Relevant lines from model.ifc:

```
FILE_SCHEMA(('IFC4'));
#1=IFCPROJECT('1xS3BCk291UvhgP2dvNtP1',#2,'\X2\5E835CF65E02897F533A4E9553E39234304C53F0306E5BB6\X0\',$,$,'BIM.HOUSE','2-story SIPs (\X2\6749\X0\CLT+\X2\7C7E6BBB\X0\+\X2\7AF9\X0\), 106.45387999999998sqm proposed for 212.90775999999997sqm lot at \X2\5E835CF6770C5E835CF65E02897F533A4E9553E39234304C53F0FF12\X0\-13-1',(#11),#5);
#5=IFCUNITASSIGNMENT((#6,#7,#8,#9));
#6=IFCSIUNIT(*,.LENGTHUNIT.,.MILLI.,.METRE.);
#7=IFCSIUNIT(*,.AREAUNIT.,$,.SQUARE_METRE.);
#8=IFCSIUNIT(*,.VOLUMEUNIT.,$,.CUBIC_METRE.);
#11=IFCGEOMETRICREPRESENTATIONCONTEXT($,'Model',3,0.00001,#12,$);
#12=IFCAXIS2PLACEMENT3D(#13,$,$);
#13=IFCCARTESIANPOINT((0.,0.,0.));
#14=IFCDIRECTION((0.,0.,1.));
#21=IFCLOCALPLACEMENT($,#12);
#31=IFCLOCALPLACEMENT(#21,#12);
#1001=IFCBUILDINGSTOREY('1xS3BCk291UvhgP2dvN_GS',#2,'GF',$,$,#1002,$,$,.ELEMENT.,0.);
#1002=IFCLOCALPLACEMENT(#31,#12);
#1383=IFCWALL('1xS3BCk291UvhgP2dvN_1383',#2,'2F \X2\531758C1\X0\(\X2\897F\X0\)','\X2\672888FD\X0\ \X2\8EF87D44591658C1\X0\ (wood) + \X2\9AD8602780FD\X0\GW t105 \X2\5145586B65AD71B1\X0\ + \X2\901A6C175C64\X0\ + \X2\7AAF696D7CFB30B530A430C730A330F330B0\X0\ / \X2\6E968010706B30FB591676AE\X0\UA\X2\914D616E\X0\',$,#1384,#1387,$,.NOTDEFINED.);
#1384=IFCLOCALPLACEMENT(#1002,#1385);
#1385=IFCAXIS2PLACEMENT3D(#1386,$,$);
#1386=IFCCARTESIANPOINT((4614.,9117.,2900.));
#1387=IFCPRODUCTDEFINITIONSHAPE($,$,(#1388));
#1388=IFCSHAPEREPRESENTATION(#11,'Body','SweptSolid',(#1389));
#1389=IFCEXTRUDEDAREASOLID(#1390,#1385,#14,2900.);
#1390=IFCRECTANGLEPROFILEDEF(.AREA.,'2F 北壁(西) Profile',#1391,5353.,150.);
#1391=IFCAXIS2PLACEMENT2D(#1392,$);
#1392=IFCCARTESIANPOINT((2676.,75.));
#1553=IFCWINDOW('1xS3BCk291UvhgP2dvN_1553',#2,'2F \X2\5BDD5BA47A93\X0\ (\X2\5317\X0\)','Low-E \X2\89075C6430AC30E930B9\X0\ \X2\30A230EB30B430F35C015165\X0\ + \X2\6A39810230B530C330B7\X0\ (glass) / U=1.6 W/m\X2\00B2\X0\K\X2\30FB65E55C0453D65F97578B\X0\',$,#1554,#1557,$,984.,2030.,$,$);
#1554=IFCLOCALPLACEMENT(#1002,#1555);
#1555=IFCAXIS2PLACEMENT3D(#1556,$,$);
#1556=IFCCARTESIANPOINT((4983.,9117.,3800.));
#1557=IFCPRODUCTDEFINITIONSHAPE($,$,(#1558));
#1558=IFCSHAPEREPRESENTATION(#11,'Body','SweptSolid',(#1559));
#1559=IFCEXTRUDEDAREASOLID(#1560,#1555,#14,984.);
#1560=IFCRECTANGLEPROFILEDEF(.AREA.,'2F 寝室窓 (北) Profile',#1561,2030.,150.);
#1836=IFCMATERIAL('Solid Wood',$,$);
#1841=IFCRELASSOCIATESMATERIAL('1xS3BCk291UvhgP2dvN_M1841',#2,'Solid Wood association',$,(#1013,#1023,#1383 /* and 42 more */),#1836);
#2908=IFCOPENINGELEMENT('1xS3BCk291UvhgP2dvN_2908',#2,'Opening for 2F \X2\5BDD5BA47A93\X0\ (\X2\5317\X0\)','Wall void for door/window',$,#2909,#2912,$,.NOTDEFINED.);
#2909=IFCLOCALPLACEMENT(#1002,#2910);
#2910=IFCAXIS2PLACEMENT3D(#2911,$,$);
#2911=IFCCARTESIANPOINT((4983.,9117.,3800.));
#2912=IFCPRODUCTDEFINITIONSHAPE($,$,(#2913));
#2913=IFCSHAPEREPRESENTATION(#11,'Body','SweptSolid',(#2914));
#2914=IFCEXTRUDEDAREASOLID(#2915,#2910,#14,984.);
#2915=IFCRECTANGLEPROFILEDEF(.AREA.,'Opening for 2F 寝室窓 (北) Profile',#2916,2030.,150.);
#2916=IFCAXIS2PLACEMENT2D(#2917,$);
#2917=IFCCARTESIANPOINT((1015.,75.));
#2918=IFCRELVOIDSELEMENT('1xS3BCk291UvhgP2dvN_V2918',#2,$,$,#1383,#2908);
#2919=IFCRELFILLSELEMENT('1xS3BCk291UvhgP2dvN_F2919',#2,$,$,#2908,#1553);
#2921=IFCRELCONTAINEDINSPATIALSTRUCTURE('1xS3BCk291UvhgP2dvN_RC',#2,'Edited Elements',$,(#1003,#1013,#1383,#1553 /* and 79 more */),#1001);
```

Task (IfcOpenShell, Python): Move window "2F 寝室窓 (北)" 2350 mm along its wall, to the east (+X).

```python
import ifcopenshell
import ifcopenshell.api.geometry
import ifcopenshell.util.placement
import ifcopenshell.util.unit

model = ifcopenshell.open("model.ifc")
unit_scale = ifcopenshell.util.unit.calculate_unit_scale(model)

window = model.by_id(1553)
opening = window.FillsVoids[0].RelatingOpeningElement
wall = opening.VoidsElements[0].RelatingBuildingElement

wall_matrix = ifcopenshell.util.placement.get_local_placement(wall.ObjectPlacement)
shift = wall_matrix[:3, 0] * 2.35 / unit_scale
before = ifcopenshell.util.placement.get_local_placement(window.ObjectPlacement)[:3, 3].copy()

# The window is not placed relative to its opening, so move both.
for product in (opening, window):
    matrix = ifcopenshell.util.placement.get_local_placement(product.ObjectPlacement)
    matrix[:3, 3] += shift
    ifcopenshell.api.geometry.edit_object_placement(model, product=product, matrix=matrix, is_si=False)

after = ifcopenshell.util.placement.get_local_placement(window.ObjectPlacement)[:3, 3]
print("window moved by", (after - before).round(3) + 0.0)

model.write("model_rev.ifc")
```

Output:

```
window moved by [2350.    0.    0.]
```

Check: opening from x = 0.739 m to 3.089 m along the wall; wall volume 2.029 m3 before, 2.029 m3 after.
